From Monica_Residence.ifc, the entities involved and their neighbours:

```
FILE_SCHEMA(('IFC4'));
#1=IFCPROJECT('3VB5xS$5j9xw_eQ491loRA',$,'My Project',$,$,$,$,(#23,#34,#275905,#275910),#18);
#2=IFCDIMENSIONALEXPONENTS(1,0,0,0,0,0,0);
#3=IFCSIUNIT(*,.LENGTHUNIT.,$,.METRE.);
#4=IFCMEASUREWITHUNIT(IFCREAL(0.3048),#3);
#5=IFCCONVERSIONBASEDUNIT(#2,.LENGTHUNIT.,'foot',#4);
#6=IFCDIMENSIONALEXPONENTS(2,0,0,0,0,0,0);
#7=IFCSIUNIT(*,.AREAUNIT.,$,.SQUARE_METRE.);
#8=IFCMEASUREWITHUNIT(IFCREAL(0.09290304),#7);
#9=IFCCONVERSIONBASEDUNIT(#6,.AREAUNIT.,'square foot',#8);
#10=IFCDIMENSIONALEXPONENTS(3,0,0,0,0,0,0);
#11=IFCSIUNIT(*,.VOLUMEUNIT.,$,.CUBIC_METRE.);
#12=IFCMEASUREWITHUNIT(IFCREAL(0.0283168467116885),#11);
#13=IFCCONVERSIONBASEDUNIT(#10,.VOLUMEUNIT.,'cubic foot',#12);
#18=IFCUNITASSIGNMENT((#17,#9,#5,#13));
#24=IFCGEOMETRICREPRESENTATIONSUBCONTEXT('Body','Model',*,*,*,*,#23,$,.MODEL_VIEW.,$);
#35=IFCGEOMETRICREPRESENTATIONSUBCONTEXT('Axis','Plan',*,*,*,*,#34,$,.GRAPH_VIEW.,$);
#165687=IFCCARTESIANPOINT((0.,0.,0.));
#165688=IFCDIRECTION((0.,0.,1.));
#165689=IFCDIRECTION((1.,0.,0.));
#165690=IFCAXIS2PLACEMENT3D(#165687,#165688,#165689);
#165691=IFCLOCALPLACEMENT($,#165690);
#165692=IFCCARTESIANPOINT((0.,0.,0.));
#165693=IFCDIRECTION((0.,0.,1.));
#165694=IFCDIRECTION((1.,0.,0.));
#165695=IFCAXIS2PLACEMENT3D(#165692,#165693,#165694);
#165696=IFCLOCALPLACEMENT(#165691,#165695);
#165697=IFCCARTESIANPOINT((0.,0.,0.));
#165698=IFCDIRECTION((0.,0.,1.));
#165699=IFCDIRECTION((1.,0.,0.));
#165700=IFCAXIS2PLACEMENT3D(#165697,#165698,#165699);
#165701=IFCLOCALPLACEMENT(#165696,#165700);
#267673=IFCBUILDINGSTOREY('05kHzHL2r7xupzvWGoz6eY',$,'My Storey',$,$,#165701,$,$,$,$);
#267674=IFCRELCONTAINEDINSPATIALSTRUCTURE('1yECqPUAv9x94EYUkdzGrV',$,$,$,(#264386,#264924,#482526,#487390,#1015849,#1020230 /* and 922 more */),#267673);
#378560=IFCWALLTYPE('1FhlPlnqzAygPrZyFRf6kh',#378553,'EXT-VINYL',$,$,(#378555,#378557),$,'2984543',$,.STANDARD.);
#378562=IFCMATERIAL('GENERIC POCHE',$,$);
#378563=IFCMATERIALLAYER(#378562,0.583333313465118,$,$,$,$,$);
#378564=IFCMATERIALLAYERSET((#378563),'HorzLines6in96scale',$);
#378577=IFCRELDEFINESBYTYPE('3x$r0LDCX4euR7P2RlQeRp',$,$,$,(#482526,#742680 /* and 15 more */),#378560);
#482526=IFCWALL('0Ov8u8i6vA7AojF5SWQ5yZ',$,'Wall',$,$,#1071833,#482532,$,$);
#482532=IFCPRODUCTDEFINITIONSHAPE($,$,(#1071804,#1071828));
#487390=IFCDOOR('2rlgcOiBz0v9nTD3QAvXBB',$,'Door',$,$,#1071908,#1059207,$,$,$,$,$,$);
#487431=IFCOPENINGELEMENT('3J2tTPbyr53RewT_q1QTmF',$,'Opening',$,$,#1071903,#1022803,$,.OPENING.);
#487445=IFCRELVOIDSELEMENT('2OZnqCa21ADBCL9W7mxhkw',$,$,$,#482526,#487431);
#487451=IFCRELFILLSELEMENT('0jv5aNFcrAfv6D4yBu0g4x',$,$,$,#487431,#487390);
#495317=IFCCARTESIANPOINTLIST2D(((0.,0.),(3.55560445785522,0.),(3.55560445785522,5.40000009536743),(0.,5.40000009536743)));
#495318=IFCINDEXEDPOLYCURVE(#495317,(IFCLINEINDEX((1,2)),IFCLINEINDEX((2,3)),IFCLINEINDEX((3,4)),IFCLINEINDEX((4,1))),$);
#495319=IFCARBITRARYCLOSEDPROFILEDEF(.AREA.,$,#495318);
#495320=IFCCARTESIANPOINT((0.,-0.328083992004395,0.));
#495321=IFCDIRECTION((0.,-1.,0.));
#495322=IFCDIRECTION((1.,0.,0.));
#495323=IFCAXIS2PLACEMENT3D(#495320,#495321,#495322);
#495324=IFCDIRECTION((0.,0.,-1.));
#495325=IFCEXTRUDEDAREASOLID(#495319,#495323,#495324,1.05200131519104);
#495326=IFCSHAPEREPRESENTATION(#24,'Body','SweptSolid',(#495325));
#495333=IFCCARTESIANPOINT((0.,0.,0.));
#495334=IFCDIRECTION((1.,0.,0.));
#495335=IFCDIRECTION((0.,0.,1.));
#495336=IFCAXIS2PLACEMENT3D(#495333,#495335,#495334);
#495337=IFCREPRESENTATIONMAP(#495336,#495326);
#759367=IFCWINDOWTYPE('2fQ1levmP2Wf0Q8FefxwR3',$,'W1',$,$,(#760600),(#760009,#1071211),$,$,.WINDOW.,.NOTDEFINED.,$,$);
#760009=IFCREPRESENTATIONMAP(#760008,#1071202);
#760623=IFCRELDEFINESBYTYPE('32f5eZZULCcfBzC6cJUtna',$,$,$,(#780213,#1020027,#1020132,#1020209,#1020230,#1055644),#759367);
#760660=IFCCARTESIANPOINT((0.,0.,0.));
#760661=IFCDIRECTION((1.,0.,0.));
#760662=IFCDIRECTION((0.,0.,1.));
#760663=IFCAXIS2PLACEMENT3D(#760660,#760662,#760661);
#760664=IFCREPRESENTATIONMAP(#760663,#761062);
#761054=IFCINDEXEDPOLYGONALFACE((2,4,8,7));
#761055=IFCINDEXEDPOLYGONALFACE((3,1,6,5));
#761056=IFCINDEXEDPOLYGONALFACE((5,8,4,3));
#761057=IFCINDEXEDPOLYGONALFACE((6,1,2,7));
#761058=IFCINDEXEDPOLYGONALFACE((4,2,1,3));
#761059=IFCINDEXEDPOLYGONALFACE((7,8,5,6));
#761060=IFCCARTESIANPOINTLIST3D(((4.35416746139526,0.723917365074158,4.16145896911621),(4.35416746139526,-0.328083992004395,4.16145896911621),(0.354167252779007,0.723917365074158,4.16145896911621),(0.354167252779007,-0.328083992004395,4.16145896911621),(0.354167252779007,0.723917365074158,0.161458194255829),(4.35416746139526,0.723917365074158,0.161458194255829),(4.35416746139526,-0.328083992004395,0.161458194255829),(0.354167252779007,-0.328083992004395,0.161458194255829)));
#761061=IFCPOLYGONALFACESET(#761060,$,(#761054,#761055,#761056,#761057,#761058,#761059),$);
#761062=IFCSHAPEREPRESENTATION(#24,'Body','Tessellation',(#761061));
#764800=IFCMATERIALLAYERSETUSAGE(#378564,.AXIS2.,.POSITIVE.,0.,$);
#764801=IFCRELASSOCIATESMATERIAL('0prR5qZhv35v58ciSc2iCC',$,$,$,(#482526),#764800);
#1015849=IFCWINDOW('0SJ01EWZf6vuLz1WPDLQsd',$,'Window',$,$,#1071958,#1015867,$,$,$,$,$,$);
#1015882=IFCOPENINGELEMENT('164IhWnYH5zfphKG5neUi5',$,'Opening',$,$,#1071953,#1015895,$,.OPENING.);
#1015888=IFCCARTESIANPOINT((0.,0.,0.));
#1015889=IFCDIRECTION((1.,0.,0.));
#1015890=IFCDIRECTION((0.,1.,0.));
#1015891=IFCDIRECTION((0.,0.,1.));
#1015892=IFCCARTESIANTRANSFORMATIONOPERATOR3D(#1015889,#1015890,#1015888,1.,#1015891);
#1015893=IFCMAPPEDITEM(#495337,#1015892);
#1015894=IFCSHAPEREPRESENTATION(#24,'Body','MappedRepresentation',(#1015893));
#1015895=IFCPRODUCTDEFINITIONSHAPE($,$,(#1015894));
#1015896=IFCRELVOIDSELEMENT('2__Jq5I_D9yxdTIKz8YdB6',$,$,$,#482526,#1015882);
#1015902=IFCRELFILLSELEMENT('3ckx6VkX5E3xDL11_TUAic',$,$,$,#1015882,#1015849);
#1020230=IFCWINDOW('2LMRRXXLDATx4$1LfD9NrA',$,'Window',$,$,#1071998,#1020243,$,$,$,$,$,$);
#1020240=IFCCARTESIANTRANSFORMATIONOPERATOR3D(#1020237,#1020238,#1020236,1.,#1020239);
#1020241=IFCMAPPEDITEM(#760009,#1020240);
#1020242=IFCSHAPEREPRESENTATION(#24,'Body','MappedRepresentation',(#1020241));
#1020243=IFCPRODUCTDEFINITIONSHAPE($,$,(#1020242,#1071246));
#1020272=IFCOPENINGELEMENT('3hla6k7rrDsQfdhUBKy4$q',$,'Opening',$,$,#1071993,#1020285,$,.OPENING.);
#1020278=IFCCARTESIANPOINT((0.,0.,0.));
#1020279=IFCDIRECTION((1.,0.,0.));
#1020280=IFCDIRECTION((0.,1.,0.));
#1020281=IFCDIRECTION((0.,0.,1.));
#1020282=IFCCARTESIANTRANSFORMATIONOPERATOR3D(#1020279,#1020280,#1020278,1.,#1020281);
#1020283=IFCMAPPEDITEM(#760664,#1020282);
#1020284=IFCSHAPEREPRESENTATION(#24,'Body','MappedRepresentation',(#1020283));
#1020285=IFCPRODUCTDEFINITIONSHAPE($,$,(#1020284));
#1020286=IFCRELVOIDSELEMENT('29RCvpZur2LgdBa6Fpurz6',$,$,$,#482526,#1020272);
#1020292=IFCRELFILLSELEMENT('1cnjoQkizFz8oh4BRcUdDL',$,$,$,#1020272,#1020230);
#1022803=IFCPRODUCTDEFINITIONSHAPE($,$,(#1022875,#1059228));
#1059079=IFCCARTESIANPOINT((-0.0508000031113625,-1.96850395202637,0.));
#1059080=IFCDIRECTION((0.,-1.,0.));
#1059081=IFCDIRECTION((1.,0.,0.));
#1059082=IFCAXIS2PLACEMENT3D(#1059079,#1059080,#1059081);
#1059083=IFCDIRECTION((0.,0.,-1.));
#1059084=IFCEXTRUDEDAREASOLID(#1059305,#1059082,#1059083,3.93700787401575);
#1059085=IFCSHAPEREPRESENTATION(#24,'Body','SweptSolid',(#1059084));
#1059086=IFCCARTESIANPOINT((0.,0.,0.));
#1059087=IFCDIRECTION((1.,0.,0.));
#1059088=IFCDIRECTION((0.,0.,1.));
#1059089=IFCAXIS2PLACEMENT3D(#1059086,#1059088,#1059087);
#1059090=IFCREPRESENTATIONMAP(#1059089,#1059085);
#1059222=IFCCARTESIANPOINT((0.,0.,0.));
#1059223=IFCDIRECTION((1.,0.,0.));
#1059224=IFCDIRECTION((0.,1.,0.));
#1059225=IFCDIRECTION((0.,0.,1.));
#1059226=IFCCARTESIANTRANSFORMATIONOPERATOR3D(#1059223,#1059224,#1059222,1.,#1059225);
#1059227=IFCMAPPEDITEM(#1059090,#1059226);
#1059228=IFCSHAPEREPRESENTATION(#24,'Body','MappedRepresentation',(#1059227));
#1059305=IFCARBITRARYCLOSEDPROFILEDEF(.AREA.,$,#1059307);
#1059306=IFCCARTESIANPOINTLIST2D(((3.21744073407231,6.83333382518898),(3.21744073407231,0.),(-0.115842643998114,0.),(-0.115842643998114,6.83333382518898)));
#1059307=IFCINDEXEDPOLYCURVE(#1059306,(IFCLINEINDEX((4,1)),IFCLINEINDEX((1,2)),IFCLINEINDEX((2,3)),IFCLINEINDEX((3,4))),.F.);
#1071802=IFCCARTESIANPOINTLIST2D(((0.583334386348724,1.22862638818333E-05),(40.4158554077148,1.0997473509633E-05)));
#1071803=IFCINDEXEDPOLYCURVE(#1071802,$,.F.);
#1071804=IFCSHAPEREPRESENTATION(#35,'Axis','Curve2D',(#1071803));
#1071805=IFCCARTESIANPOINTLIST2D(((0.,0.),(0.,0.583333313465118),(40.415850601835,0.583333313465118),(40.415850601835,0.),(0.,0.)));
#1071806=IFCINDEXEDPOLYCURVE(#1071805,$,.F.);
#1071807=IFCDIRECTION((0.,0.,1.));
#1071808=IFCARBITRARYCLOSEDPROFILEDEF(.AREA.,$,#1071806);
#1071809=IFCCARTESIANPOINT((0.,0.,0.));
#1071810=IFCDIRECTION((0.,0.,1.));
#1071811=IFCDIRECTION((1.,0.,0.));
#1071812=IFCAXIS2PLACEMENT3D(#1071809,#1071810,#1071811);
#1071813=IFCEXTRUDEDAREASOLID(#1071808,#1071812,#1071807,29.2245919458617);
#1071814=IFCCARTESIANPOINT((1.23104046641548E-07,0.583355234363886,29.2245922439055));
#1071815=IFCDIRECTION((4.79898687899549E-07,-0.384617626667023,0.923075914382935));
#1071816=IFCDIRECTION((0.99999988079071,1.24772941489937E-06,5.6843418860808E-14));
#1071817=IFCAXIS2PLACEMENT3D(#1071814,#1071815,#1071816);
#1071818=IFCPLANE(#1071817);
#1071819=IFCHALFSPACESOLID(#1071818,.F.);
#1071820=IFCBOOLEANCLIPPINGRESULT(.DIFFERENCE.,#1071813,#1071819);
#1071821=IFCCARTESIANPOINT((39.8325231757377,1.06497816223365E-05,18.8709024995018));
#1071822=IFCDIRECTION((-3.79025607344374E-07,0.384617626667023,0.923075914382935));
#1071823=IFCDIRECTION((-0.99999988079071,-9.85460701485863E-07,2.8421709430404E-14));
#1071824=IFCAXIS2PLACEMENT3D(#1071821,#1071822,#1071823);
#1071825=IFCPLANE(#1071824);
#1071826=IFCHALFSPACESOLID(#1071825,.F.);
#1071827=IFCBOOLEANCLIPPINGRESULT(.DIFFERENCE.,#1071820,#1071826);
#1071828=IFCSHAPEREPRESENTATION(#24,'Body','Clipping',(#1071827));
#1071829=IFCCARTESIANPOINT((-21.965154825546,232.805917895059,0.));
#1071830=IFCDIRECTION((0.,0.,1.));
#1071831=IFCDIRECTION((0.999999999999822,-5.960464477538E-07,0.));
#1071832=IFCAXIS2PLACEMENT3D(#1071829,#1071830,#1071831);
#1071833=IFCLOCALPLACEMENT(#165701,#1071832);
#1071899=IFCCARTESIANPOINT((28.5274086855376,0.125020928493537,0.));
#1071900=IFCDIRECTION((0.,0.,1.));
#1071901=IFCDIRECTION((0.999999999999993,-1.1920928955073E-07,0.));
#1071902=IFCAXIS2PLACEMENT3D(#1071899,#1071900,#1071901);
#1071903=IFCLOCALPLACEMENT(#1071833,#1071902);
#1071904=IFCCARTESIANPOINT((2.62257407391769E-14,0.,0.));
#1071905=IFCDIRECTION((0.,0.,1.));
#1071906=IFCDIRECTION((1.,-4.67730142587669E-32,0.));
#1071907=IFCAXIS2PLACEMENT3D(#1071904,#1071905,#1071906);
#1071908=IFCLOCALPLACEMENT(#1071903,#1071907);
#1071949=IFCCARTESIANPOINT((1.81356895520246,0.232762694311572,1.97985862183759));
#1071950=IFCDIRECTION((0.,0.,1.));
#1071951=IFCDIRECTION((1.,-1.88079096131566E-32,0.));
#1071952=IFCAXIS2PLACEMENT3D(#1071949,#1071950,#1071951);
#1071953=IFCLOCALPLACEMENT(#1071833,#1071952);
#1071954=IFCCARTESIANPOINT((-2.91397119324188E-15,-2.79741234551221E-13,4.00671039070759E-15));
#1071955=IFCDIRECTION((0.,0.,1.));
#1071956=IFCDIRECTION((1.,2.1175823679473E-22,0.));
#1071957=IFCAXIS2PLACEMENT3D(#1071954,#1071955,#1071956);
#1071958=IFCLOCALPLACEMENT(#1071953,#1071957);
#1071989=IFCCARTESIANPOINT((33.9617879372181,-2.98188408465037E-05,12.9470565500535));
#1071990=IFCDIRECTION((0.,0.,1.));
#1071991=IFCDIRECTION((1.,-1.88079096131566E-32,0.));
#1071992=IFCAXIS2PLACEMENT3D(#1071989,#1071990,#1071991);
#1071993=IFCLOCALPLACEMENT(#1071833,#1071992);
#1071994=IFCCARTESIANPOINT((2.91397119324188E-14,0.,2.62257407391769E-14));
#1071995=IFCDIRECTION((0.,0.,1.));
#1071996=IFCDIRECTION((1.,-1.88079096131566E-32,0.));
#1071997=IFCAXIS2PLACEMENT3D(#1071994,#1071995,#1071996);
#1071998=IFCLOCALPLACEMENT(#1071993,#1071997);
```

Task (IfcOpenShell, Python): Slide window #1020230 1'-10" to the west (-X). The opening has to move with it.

```python
import ifcopenshell
import ifcopenshell.api.geometry
import ifcopenshell.util.placement
import ifcopenshell.util.unit

model = ifcopenshell.open("Monica_Residence.ifc")
unit_scale = ifcopenshell.util.unit.calculate_unit_scale(model)

window = model.by_guid("2LMRRXXLDATx4$1LfD9NrA")
opening = window.FillsVoids[0].RelatingOpeningElement
wall = opening.VoidsElements[0].RelatingBuildingElement

wall_matrix = ifcopenshell.util.placement.get_local_placement(wall.ObjectPlacement)
shift = wall_matrix[:3, 0] * -22 * 0.0254 / unit_scale
before = ifcopenshell.util.placement.get_local_placement(window.ObjectPlacement)[:3, 3].copy()

# The window is placed relative to its opening, so it follows when the opening moves.
matrix = ifcopenshell.util.placement.get_local_placement(opening.ObjectPlacement)
matrix[:3, 3] += shift
ifcopenshell.api.geometry.edit_object_placement(
    model, product=opening, matrix=matrix, is_si=False, should_transform_children=True
)

after = ifcopenshell.util.placement.get_local_placement(window.ObjectPlacement)[:3, 3]
print("window moved by", (after - before).round(3) + 0.0)

model.write("Monica_Residence_updated.ifc")
```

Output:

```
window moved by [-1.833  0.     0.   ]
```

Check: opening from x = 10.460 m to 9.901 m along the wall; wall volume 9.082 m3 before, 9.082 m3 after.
